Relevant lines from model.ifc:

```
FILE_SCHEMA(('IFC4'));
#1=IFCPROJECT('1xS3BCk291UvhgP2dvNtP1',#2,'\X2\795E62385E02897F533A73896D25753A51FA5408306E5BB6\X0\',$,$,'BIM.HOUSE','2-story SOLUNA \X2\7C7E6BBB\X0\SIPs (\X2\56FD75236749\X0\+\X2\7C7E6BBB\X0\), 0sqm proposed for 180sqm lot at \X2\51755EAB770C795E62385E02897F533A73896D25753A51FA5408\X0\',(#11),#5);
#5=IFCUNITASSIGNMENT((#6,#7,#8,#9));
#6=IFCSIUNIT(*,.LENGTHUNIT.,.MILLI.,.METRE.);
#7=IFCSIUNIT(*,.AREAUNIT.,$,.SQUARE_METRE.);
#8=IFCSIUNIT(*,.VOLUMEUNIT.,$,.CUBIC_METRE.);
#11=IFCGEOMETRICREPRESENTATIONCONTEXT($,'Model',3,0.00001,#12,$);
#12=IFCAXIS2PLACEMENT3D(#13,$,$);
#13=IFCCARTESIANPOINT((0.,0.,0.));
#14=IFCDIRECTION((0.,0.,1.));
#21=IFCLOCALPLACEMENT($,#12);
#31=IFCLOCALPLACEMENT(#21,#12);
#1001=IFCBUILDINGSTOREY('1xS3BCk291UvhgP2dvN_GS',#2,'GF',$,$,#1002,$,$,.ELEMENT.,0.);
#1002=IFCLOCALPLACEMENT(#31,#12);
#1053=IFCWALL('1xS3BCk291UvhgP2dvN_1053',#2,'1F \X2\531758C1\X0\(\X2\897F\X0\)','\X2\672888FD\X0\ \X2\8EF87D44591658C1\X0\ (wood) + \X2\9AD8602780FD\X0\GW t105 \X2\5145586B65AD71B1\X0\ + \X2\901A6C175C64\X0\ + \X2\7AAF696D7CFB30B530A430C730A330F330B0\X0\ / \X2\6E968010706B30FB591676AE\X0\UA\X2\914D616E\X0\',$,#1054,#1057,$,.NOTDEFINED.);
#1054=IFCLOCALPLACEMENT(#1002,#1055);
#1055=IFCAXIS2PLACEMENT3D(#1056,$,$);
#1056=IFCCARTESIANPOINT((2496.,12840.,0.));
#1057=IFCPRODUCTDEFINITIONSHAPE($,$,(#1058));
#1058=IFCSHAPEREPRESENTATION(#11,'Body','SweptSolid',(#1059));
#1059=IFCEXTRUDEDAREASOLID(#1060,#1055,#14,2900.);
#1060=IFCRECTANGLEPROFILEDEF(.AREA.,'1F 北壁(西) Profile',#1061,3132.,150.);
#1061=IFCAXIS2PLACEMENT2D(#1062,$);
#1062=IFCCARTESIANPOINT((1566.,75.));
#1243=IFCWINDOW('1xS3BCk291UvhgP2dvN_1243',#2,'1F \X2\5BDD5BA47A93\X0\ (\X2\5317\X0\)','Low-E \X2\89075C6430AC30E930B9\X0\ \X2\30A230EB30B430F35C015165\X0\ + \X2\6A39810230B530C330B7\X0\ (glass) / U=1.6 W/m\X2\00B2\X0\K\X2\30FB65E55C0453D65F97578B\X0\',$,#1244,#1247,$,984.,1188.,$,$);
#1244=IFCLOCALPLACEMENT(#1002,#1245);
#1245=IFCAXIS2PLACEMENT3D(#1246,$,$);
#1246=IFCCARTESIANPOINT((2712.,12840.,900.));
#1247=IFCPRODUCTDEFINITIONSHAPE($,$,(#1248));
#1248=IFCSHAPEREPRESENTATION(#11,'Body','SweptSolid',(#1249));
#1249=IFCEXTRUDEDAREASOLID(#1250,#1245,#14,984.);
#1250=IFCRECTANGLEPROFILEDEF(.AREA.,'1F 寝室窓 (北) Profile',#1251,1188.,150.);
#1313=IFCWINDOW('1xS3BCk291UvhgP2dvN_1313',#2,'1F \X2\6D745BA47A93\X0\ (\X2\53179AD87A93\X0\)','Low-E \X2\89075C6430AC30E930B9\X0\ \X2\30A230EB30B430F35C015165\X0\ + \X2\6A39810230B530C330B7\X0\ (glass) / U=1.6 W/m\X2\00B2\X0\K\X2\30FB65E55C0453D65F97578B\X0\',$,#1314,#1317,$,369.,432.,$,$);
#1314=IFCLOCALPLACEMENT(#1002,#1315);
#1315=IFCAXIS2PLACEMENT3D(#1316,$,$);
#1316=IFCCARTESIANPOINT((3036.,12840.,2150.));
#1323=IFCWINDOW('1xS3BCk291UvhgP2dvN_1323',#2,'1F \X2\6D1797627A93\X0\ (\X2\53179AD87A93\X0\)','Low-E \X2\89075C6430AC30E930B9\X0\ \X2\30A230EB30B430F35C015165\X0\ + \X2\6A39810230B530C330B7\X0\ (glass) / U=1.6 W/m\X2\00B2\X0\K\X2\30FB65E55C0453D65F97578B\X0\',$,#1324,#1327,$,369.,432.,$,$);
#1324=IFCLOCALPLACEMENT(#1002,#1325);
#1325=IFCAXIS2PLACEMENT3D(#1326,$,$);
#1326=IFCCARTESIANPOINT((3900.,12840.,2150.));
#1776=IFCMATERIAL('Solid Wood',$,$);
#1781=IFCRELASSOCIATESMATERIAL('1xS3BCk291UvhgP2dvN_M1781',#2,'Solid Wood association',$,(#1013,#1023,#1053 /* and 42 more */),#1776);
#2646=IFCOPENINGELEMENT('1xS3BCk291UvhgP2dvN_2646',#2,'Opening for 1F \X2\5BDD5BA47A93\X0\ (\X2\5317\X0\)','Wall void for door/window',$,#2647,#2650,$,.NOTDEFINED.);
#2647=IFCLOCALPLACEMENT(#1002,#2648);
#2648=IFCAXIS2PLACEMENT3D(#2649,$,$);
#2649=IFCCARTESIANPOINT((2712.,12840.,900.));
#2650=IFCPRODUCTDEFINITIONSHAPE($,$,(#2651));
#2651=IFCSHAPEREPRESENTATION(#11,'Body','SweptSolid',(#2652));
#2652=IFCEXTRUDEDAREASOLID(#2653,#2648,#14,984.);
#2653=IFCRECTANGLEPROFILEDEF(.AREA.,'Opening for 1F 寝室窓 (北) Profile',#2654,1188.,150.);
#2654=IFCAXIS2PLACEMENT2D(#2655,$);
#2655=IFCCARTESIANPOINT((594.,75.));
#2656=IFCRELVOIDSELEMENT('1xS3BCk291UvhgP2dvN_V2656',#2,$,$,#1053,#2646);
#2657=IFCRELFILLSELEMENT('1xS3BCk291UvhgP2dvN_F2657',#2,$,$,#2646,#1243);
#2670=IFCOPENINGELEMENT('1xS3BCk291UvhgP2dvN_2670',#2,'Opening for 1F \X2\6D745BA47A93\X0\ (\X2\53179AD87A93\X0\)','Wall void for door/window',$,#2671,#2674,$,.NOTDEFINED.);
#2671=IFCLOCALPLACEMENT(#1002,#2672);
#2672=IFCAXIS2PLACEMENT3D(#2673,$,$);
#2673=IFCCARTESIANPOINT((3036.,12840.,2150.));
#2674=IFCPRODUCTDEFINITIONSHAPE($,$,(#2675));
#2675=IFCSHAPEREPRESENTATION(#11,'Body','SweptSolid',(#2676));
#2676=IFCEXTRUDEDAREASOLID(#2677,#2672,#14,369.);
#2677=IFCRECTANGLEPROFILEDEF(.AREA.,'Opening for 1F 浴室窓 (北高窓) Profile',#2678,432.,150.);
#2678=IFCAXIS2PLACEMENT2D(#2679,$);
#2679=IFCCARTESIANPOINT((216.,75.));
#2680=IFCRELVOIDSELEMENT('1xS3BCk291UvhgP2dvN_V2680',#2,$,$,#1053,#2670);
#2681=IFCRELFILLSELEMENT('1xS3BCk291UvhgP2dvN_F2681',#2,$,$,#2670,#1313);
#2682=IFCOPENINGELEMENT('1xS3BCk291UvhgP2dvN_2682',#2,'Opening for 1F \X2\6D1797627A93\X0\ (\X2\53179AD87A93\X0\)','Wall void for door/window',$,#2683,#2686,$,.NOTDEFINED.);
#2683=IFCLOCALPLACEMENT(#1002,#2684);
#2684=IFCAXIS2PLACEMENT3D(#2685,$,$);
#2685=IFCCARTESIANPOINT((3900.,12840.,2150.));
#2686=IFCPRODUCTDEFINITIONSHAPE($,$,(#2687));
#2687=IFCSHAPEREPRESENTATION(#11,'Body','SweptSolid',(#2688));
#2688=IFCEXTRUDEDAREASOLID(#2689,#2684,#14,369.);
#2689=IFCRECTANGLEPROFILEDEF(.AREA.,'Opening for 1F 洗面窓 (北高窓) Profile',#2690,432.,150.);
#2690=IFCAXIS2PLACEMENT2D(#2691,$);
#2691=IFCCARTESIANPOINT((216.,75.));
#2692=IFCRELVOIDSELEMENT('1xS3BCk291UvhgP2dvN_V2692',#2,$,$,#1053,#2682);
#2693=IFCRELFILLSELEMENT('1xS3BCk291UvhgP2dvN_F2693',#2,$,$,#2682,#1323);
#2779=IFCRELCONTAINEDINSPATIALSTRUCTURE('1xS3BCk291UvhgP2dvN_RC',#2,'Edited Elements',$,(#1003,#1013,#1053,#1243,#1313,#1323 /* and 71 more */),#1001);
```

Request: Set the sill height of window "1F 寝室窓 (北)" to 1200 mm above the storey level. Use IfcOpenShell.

```python
import numpy as np
import ifcopenshell
import ifcopenshell.api.geometry
import ifcopenshell.geom
import ifcopenshell.util.element
import ifcopenshell.util.placement
import ifcopenshell.util.shape
import ifcopenshell.util.unit

model = ifcopenshell.open("model.ifc")
unit_scale = ifcopenshell.util.unit.calculate_unit_scale(model)

window = model.by_guid("1xS3BCk291UvhgP2dvN_1243")
opening = window.FillsVoids[0].RelatingOpeningElement
storey = ifcopenshell.util.element.get_container(window, ifc_class="IfcBuildingStorey")
level = ifcopenshell.util.placement.get_local_placement(storey.ObjectPlacement)[2, 3]

# The opening's origin need not be at the sill, so measure its lowest point.
shape = ifcopenshell.geom.create_shape(ifcopenshell.geom.settings(), opening)
bottom = ifcopenshell.util.shape.get_shape_bottom_elevation(shape, shape.geometry) / unit_scale
dz = level + 1200.0 - bottom

shift = np.array([0.0, 0.0, dz])
# The window is not placed relative to its opening, so move both.
for product in (opening, window):
    matrix = ifcopenshell.util.placement.get_local_placement(product.ObjectPlacement)
    matrix[:3, 3] += shift
    ifcopenshell.api.geometry.edit_object_placement(model, product=product, matrix=matrix, is_si=False)

print(f"moved by {dz * unit_scale:+.3f} m")

model.write("model_v2.ifc")
```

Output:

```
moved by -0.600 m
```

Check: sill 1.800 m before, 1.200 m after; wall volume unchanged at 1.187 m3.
